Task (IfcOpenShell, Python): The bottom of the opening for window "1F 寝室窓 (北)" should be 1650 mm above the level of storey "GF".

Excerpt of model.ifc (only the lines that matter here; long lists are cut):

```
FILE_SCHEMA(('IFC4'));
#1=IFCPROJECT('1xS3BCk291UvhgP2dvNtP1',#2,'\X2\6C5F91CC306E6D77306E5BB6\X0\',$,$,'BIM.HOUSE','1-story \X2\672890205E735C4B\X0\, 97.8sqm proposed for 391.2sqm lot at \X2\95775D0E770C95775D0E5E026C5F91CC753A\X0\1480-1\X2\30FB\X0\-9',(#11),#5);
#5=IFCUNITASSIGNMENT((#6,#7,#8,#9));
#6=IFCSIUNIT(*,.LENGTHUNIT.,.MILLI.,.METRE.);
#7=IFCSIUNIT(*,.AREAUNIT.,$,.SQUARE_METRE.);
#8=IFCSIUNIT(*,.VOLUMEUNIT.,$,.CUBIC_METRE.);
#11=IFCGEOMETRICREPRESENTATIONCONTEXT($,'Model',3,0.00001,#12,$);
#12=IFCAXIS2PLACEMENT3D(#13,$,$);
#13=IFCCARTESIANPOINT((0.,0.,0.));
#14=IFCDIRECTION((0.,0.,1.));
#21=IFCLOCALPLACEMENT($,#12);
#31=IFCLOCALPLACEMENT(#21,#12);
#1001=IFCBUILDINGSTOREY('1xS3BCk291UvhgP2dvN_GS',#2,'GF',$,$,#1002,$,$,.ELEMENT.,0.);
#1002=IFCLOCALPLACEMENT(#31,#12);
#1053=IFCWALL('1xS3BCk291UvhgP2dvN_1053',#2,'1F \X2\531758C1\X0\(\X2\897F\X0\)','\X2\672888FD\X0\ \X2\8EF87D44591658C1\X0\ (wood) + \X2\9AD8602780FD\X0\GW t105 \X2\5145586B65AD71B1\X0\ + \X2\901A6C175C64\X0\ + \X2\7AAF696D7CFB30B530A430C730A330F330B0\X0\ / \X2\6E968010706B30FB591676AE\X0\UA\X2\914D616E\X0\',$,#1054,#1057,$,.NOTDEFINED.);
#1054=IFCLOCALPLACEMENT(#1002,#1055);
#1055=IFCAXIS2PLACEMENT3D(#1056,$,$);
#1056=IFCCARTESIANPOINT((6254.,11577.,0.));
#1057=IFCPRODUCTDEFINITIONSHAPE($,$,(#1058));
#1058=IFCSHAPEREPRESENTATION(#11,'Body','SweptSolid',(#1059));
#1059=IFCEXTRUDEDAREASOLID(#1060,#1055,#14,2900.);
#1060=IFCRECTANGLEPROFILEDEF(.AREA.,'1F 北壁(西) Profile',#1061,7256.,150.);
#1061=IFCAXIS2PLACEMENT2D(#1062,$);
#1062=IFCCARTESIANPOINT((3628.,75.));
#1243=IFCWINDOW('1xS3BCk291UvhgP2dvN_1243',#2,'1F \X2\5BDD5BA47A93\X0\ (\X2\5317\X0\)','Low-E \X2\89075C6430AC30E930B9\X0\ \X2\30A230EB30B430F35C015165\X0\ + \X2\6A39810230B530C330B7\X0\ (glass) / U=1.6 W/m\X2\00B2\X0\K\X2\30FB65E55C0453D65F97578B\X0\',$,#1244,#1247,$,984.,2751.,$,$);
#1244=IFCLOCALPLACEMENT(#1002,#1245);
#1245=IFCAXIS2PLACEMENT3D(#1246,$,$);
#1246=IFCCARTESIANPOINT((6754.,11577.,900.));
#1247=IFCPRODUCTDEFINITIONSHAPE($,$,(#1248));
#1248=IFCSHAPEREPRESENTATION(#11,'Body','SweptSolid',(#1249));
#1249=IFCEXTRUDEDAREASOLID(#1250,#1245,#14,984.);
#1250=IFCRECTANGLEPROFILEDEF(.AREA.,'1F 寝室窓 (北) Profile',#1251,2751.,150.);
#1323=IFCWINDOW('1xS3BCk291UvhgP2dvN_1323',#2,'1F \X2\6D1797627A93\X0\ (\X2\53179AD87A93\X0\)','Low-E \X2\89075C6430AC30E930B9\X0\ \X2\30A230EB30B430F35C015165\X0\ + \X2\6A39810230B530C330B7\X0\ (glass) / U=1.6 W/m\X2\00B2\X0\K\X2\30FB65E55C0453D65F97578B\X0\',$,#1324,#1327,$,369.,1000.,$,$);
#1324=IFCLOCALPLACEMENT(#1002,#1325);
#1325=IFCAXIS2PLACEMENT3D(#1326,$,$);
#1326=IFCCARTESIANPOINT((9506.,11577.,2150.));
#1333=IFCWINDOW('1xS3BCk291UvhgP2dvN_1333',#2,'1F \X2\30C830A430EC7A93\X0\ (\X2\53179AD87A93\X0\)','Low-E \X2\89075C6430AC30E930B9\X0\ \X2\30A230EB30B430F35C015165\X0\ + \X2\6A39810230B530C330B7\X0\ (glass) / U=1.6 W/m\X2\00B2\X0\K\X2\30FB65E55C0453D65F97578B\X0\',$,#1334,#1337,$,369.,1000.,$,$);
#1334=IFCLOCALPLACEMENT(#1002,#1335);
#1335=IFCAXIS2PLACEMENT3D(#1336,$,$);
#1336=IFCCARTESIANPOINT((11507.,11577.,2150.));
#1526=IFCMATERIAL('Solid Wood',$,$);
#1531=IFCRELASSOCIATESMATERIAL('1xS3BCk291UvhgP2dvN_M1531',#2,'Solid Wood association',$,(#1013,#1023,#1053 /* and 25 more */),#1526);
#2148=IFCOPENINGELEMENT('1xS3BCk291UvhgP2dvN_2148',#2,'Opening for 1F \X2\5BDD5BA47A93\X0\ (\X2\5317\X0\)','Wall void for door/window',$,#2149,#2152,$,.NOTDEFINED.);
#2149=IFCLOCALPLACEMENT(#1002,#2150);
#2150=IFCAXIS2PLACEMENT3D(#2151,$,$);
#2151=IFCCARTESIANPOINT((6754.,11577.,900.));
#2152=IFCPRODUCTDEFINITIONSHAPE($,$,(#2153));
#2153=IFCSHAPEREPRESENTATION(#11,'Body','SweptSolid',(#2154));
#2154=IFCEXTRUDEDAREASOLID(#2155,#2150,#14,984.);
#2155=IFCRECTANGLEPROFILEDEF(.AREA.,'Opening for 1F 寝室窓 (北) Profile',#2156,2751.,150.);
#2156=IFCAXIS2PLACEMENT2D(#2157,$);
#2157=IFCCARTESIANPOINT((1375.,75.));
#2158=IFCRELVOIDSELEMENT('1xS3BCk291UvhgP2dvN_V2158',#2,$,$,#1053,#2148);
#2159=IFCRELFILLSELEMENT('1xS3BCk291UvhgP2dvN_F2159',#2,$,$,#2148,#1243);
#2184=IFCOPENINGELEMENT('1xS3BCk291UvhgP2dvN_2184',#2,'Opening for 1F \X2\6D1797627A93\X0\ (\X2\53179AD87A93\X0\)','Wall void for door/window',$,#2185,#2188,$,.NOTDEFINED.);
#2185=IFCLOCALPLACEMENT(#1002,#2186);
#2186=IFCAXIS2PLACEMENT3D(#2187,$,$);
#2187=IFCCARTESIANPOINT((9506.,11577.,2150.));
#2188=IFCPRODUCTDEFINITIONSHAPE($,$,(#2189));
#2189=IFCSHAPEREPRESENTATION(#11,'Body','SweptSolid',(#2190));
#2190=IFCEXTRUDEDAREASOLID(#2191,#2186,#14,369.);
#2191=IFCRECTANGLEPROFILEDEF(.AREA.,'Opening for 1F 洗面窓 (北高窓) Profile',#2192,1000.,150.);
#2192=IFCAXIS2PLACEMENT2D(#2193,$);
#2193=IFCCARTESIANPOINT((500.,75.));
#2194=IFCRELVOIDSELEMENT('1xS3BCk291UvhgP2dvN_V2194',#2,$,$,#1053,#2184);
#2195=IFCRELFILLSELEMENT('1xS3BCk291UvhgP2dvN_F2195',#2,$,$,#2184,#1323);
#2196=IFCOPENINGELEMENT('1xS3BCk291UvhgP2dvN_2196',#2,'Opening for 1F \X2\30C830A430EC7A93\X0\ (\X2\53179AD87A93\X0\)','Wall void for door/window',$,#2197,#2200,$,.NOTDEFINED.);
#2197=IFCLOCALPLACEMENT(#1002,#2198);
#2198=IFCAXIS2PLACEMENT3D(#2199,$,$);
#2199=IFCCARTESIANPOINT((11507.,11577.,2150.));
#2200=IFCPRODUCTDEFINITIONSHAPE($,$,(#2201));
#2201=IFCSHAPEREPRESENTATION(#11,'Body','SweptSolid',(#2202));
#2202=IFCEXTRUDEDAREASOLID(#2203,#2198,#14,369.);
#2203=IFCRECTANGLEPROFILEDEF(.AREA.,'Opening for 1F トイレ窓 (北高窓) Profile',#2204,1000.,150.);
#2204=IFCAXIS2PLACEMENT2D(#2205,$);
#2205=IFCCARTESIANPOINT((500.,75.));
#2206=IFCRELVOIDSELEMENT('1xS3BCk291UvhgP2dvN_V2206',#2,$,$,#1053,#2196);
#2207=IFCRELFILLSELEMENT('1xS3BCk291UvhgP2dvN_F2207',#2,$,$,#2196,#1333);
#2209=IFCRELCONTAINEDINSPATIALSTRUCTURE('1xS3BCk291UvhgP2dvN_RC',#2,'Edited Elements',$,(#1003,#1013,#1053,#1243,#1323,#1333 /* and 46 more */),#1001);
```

```python
import numpy as np
import ifcopenshell
import ifcopenshell.api.geometry
import ifcopenshell.geom
import ifcopenshell.util.element
import ifcopenshell.util.placement
import ifcopenshell.util.shape
import ifcopenshell.util.unit

model = ifcopenshell.open("model.ifc")
unit_scale = ifcopenshell.util.unit.calculate_unit_scale(model)

window = model.by_guid("1xS3BCk291UvhgP2dvN_1243")
opening = window.FillsVoids[0].RelatingOpeningElement
storey = ifcopenshell.util.element.get_container(window, ifc_class="IfcBuildingStorey")
level = ifcopenshell.util.placement.get_local_placement(storey.ObjectPlacement)[2, 3]

# The opening's origin need not be at the sill, so measure its lowest point.
shape = ifcopenshell.geom.create_shape(ifcopenshell.geom.settings(), opening)
bottom = ifcopenshell.util.shape.get_shape_bottom_elevation(shape, shape.geometry) / unit_scale
dz = level + 1.65 / unit_scale - bottom

shift = np.array([0.0, 0.0, dz])
# The window is not placed relative to its opening, so move both.
for product in (opening, window):
    matrix = ifcopenshell.util.placement.get_local_placement(product.ObjectPlacement)
    matrix[:3, 3] += shift
    ifcopenshell.api.geometry.edit_object_placement(model, product=product, matrix=matrix, is_si=False)

print(f"moved by {dz * unit_scale:+.3f} m")

model.write("model_v2.ifc")
```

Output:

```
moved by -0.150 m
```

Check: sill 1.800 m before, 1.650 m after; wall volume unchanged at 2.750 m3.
